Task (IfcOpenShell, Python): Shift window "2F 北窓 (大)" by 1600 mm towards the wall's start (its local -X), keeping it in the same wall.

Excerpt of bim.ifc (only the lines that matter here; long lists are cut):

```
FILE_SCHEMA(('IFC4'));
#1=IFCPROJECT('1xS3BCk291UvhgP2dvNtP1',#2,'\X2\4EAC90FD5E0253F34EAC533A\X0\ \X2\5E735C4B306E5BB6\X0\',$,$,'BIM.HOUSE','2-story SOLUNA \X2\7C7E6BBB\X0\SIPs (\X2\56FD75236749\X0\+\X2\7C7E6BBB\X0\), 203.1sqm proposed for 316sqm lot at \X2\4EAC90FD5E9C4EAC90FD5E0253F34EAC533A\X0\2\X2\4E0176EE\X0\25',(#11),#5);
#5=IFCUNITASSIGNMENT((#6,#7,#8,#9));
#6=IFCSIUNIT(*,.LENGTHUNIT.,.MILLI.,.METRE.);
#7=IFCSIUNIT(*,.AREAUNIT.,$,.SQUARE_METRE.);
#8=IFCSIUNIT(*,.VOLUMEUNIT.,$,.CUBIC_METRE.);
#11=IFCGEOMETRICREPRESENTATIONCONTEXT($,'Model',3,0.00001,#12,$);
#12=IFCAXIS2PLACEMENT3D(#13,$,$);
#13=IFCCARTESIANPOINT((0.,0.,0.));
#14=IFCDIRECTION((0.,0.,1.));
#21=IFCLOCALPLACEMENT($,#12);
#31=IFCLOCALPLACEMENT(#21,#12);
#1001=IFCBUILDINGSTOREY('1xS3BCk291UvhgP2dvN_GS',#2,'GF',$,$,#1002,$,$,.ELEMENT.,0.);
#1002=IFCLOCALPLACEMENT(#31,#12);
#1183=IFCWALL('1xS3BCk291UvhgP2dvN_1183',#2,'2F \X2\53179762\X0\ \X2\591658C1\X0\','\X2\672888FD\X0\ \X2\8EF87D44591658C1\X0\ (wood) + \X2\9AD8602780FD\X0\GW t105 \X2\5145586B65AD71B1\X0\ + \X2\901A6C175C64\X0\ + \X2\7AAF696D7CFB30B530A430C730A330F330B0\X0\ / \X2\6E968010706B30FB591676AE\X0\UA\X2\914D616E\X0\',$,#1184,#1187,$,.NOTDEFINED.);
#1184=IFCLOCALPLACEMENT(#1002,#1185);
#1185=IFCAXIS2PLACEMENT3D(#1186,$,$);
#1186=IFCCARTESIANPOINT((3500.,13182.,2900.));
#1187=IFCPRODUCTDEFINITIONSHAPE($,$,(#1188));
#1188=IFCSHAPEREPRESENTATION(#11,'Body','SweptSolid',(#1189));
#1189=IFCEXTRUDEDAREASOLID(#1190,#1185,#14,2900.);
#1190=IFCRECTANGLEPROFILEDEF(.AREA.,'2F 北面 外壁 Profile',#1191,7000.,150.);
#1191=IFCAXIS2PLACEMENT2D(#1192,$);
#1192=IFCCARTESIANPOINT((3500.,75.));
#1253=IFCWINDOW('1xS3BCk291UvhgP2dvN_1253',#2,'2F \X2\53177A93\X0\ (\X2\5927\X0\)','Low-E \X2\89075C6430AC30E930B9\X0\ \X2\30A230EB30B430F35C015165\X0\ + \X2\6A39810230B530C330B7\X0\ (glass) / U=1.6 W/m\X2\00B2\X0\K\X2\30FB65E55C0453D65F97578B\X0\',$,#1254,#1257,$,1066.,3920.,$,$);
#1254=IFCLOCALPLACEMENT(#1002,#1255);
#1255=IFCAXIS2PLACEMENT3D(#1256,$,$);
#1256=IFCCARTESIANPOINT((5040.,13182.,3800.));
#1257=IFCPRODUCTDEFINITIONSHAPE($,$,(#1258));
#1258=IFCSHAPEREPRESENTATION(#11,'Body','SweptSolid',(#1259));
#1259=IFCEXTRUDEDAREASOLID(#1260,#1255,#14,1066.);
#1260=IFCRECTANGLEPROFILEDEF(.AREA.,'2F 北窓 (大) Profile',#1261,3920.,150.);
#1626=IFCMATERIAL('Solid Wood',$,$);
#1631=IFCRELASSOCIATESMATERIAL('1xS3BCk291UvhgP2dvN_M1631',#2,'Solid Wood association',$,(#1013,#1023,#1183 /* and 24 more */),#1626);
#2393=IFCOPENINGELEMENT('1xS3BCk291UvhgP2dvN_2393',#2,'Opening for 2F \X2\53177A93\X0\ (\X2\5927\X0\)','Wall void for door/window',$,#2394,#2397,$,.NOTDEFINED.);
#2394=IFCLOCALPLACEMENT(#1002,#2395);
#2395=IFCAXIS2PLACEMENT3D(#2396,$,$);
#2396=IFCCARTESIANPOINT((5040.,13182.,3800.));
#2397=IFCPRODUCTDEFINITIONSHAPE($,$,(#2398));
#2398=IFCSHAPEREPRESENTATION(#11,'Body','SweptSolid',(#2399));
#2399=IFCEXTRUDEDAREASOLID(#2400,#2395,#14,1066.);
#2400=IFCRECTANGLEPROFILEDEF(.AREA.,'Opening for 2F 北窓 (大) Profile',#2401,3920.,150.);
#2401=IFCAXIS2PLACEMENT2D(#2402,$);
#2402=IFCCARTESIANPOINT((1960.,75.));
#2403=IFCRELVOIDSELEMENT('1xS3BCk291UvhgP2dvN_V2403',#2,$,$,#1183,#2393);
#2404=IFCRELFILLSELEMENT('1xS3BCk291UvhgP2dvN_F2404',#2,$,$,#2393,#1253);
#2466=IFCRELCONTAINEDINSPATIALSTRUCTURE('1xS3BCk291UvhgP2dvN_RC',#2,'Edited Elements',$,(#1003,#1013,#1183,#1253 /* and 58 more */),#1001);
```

```python
import ifcopenshell
import ifcopenshell.api.geometry
import ifcopenshell.util.placement
import ifcopenshell.util.unit

model = ifcopenshell.open("bim.ifc")
unit_scale = ifcopenshell.util.unit.calculate_unit_scale(model)

window = model.by_guid("1xS3BCk291UvhgP2dvN_1253")
opening = window.FillsVoids[0].RelatingOpeningElement
wall = opening.VoidsElements[0].RelatingBuildingElement

wall_matrix = ifcopenshell.util.placement.get_local_placement(wall.ObjectPlacement)
shift = wall_matrix[:3, 0] * -1.6 / unit_scale
before = ifcopenshell.util.placement.get_local_placement(window.ObjectPlacement)[:3, 3].copy()

# The window is not placed relative to its opening, so move both.
for product in (opening, window):
    matrix = ifcopenshell.util.placement.get_local_placement(product.ObjectPlacement)
    matrix[:3, 3] += shift
    ifcopenshell.api.geometry.edit_object_placement(model, product=product, matrix=matrix, is_si=False)

after = ifcopenshell.util.placement.get_local_placement(window.ObjectPlacement)[:3, 3]
print("window moved by", (after - before).round(3) + 0.0)

model.write("bim_edited.ifc")
```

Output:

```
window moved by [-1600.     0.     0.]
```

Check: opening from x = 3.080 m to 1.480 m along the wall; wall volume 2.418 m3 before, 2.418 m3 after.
